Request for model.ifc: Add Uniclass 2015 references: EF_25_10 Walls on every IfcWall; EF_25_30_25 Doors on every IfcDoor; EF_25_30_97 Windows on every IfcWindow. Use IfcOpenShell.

First a look at what the model holds.

```python
import ifcopenshell

model = ifcopenshell.open("model.ifc")
print(model.schema)
print("classifications:", [c.Name for c in model.by_type("IfcClassification")])
for ifc_class in ("IfcDoor", "IfcRoof", "IfcStair", "IfcWall", "IfcWindow"):
    print(ifc_class, len(model.by_type(ifc_class)))
```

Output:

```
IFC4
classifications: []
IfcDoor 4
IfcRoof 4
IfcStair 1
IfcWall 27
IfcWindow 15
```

```python
import ifcopenshell
import ifcopenshell.api.classification

model = ifcopenshell.open("model.ifc")

system = ifcopenshell.api.classification.add_classification(model, classification="Uniclass 2015")

codes = {
    "IfcWall": ("EF_25_10", "Walls"),
    "IfcDoor": ("EF_25_30_25", "Doors"),
    "IfcWindow": ("EF_25_30_97", "Windows"),
}
for ifc_class, (code, name) in codes.items():
    products = model.by_type(ifc_class)
    ifcopenshell.api.classification.add_reference(
        model, products=products, classification=system, identification=code, name=name
    )
    print(code, len(products))

model.write("model_updated.ifc")
```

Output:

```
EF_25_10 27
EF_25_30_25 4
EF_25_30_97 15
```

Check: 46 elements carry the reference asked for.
